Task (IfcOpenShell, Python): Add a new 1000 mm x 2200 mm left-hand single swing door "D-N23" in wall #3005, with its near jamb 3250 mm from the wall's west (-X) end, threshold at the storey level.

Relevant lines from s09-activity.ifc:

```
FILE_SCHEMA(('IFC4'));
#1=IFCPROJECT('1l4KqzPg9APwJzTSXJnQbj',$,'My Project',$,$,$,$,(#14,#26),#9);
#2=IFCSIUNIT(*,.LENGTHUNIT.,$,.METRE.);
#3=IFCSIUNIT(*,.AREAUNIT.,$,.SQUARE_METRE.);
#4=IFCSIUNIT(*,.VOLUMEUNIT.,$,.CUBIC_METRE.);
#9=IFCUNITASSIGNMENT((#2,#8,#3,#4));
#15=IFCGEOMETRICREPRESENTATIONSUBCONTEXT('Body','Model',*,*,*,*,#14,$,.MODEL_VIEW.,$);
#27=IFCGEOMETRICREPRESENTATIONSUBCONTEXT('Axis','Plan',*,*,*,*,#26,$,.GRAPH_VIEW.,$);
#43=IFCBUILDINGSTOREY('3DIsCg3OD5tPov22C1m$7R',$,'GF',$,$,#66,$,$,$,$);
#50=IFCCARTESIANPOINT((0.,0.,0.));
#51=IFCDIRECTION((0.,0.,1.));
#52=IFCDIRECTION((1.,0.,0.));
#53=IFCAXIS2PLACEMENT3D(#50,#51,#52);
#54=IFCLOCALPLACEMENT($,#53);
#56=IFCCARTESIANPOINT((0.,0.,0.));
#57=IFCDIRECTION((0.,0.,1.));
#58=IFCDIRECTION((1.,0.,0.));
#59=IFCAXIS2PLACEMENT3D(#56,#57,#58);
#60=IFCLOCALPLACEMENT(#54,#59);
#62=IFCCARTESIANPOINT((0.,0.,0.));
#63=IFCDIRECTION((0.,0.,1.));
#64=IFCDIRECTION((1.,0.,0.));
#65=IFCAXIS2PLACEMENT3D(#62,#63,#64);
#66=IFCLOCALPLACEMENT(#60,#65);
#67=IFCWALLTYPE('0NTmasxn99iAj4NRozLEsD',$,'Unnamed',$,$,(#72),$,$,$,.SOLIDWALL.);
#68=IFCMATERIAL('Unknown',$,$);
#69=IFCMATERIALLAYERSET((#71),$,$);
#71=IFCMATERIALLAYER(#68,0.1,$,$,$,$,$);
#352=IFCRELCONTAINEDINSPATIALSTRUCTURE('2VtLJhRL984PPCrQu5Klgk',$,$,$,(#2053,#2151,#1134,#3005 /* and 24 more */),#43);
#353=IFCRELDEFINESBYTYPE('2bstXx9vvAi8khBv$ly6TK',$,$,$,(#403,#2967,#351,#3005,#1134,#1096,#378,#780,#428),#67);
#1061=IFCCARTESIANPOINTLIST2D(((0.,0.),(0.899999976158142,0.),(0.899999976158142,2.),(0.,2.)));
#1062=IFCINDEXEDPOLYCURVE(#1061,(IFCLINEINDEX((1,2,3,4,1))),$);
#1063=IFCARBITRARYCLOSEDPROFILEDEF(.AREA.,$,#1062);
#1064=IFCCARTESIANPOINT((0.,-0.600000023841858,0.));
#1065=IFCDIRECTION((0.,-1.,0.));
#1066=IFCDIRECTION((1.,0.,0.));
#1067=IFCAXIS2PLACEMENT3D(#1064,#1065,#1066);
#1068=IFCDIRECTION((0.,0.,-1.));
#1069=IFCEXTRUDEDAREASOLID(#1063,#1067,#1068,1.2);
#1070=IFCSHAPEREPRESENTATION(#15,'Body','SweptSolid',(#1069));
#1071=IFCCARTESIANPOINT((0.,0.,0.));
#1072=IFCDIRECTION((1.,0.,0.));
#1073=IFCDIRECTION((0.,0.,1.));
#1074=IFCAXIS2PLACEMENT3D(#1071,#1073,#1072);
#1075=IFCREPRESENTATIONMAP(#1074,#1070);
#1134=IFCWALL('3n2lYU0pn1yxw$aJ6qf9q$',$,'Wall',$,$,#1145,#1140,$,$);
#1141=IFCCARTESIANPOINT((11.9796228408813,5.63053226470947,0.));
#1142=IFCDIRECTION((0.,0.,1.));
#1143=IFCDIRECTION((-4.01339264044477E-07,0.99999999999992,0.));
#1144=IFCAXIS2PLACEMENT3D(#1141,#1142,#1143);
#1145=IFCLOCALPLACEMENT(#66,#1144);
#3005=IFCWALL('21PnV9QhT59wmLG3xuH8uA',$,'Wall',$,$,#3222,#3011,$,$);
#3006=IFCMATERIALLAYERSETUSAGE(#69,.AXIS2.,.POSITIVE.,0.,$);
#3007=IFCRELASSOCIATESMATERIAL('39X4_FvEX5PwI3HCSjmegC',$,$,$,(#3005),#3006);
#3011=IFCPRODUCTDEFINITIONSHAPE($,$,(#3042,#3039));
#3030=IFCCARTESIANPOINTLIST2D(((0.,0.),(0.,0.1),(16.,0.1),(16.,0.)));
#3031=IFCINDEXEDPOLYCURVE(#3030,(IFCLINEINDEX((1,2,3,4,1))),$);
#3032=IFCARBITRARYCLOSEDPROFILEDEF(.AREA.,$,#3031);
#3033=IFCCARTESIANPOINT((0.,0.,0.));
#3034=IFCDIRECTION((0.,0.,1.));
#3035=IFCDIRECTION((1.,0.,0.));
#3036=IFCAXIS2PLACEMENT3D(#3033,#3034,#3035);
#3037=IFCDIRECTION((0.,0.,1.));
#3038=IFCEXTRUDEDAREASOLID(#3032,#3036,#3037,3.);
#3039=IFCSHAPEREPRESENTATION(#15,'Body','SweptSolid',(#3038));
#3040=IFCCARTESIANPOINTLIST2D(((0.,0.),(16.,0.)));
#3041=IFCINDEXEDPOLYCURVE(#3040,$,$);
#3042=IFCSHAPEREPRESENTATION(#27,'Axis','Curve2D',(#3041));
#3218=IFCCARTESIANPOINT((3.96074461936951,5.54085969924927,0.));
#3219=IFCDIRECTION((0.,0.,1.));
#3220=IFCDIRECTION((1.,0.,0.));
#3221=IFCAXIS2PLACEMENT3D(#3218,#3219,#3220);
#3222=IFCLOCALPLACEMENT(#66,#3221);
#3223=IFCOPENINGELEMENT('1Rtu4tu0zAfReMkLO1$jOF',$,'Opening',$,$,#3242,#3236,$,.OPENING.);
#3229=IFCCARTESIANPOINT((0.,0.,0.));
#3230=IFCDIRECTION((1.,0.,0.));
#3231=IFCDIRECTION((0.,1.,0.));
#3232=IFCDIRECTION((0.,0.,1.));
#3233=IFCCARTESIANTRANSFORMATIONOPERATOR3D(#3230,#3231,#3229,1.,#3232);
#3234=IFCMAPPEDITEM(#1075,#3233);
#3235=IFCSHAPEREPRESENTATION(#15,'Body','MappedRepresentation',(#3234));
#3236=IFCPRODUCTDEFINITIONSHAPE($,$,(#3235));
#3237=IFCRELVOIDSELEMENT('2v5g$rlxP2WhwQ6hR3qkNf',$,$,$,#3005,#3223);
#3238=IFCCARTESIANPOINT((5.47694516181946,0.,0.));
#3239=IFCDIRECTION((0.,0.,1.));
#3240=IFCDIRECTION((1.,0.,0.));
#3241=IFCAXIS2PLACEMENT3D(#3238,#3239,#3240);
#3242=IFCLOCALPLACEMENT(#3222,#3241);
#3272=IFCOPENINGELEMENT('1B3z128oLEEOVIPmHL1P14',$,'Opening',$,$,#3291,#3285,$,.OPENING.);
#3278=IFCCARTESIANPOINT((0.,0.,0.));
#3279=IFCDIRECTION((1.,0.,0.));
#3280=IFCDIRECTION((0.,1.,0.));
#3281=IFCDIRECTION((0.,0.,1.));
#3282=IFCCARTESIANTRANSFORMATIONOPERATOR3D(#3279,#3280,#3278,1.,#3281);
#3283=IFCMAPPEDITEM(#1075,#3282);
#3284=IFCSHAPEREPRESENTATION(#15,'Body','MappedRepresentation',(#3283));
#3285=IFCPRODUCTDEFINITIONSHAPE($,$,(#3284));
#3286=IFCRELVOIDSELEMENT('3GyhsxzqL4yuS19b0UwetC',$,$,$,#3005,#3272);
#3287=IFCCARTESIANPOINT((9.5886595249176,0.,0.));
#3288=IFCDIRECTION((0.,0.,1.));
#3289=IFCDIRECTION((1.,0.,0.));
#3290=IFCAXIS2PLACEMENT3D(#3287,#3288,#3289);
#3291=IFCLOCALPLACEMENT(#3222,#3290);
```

```python
import numpy as np
import ifcopenshell
import ifcopenshell.api.feature
import ifcopenshell.api.geometry
import ifcopenshell.api.root
import ifcopenshell.api.spatial
import ifcopenshell.geom
import ifcopenshell.util.element
import ifcopenshell.util.placement
import ifcopenshell.util.representation
import ifcopenshell.util.shape
import ifcopenshell.util.unit

model = ifcopenshell.open("s09-activity.ifc")
unit_scale = ifcopenshell.util.unit.calculate_unit_scale(model)
settings = ifcopenshell.geom.settings()


def volume(element):
    """Net volume in cubic metres, openings subtracted."""
    shape = ifcopenshell.geom.create_shape(settings, element)
    return ifcopenshell.util.shape.get_volume(shape.geometry)


wall = model.by_guid("21PnV9QhT59wmLG3xuH8uA")
storey = ifcopenshell.util.element.get_container(wall, ifc_class="IfcBuildingStorey")
context = ifcopenshell.util.representation.get_context(model, "Model", "Body", "MODEL_VIEW")
before = volume(wall)

width, height, from_end, sill = 1, 2.2, 3.25, 0.0  # metres

# The wall runs along its own X axis, and the end named is its -X end.
wall_shape = ifcopenshell.geom.create_shape(settings, wall)
x, y, z = ifcopenshell.util.shape.get_vertices(wall_shape.geometry).T
start = x.min() + from_end
face, thickness = float(y.min()), float(y.max() - y.min())
wall_matrix = ifcopenshell.util.placement.get_local_placement(wall.ObjectPlacement)
level = ifcopenshell.util.placement.get_local_placement(storey.ObjectPlacement)[2, 3]


def in_wall(x, y):
    """Placement at x, y metres in the wall's axes, at sill height."""
    matrix = wall_matrix.copy()
    matrix[:, 3] = wall_matrix @ np.array([x / unit_scale, y / unit_scale, 0.0, 1.0])
    matrix[2, 3] = level + sill / unit_scale
    return matrix


# Opening: a box that overshoots both wall faces by 50 mm.
opening = ifcopenshell.api.root.create_entity(model, ifc_class="IfcOpeningElement", predefined_type="OPENING")
box = ifcopenshell.api.geometry.add_wall_representation(
    model, context=context, length=width, height=height, thickness=thickness + 0.1
)
ifcopenshell.api.geometry.assign_representation(model, product=opening, representation=box)
ifcopenshell.api.geometry.edit_object_placement(model, product=opening, matrix=in_wall(start, face - 0.05), is_si=False)
ifcopenshell.api.feature.add_feature(model, feature=opening, element=wall)

door = ifcopenshell.api.root.create_entity(model, ifc_class="IfcDoor", name="D-N23", predefined_type="DOOR")
door.OverallWidth, door.OverallHeight = width / unit_scale, height / unit_scale
door.OperationType = "SINGLE_SWING_LEFT"
body = ifcopenshell.api.geometry.add_door_representation(
    model,
    context=context,
    overall_width=door.OverallWidth,
    overall_height=door.OverallHeight,
    operation_type="SINGLE_SWING_LEFT",
    lining_properties={"LiningDepth": thickness / unit_scale, "ThresholdDepth": thickness / unit_scale},
)
ifcopenshell.api.geometry.assign_representation(model, product=door, representation=body)
ifcopenshell.api.spatial.assign_container(model, products=[door], relating_structure=storey)
ifcopenshell.api.feature.add_filling(model, opening=opening, element=door)

# The lining spans the wall, so the door starts at the wall face.
ifcopenshell.api.geometry.edit_object_placement(model, product=door, matrix=in_wall(start, face), is_si=False)

after = volume(wall)

print(f"wall volume {before:.3f} -> {after:.3f} m3")

model.write("s09-activity_v2.ifc")
```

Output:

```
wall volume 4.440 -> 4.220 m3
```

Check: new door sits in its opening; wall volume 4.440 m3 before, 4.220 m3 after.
